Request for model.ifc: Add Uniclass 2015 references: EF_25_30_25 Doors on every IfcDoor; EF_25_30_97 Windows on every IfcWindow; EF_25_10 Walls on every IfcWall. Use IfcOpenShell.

First a look at what the model holds.

```python
import ifcopenshell

model = ifcopenshell.open("model.ifc")
print(model.schema)
print("classifications:", [c.Name for c in model.by_type("IfcClassification")])
for ifc_class in ("IfcDoor", "IfcRoof", "IfcStair", "IfcWall", "IfcWindow"):
    print(ifc_class, len(model.by_type(ifc_class)))
```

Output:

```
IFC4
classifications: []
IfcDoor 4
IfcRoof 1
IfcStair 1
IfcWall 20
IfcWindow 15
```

```python
import ifcopenshell
import ifcopenshell.api.classification

model = ifcopenshell.open("model.ifc")

system = ifcopenshell.api.classification.add_classification(model, classification="Uniclass 2015")

codes = {
    "IfcDoor": ("EF_25_30_25", "Doors"),
    "IfcWindow": ("EF_25_30_97", "Windows"),
    "IfcWall": ("EF_25_10", "Walls"),
}
for ifc_class, (code, name) in codes.items():
    products = model.by_type(ifc_class)
    ifcopenshell.api.classification.add_reference(
        model, products=products, classification=system, identification=code, name=name
    )
    print(code, len(products))

model.write("model_rev.ifc")
```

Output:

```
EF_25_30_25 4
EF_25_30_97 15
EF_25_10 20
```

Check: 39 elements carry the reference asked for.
